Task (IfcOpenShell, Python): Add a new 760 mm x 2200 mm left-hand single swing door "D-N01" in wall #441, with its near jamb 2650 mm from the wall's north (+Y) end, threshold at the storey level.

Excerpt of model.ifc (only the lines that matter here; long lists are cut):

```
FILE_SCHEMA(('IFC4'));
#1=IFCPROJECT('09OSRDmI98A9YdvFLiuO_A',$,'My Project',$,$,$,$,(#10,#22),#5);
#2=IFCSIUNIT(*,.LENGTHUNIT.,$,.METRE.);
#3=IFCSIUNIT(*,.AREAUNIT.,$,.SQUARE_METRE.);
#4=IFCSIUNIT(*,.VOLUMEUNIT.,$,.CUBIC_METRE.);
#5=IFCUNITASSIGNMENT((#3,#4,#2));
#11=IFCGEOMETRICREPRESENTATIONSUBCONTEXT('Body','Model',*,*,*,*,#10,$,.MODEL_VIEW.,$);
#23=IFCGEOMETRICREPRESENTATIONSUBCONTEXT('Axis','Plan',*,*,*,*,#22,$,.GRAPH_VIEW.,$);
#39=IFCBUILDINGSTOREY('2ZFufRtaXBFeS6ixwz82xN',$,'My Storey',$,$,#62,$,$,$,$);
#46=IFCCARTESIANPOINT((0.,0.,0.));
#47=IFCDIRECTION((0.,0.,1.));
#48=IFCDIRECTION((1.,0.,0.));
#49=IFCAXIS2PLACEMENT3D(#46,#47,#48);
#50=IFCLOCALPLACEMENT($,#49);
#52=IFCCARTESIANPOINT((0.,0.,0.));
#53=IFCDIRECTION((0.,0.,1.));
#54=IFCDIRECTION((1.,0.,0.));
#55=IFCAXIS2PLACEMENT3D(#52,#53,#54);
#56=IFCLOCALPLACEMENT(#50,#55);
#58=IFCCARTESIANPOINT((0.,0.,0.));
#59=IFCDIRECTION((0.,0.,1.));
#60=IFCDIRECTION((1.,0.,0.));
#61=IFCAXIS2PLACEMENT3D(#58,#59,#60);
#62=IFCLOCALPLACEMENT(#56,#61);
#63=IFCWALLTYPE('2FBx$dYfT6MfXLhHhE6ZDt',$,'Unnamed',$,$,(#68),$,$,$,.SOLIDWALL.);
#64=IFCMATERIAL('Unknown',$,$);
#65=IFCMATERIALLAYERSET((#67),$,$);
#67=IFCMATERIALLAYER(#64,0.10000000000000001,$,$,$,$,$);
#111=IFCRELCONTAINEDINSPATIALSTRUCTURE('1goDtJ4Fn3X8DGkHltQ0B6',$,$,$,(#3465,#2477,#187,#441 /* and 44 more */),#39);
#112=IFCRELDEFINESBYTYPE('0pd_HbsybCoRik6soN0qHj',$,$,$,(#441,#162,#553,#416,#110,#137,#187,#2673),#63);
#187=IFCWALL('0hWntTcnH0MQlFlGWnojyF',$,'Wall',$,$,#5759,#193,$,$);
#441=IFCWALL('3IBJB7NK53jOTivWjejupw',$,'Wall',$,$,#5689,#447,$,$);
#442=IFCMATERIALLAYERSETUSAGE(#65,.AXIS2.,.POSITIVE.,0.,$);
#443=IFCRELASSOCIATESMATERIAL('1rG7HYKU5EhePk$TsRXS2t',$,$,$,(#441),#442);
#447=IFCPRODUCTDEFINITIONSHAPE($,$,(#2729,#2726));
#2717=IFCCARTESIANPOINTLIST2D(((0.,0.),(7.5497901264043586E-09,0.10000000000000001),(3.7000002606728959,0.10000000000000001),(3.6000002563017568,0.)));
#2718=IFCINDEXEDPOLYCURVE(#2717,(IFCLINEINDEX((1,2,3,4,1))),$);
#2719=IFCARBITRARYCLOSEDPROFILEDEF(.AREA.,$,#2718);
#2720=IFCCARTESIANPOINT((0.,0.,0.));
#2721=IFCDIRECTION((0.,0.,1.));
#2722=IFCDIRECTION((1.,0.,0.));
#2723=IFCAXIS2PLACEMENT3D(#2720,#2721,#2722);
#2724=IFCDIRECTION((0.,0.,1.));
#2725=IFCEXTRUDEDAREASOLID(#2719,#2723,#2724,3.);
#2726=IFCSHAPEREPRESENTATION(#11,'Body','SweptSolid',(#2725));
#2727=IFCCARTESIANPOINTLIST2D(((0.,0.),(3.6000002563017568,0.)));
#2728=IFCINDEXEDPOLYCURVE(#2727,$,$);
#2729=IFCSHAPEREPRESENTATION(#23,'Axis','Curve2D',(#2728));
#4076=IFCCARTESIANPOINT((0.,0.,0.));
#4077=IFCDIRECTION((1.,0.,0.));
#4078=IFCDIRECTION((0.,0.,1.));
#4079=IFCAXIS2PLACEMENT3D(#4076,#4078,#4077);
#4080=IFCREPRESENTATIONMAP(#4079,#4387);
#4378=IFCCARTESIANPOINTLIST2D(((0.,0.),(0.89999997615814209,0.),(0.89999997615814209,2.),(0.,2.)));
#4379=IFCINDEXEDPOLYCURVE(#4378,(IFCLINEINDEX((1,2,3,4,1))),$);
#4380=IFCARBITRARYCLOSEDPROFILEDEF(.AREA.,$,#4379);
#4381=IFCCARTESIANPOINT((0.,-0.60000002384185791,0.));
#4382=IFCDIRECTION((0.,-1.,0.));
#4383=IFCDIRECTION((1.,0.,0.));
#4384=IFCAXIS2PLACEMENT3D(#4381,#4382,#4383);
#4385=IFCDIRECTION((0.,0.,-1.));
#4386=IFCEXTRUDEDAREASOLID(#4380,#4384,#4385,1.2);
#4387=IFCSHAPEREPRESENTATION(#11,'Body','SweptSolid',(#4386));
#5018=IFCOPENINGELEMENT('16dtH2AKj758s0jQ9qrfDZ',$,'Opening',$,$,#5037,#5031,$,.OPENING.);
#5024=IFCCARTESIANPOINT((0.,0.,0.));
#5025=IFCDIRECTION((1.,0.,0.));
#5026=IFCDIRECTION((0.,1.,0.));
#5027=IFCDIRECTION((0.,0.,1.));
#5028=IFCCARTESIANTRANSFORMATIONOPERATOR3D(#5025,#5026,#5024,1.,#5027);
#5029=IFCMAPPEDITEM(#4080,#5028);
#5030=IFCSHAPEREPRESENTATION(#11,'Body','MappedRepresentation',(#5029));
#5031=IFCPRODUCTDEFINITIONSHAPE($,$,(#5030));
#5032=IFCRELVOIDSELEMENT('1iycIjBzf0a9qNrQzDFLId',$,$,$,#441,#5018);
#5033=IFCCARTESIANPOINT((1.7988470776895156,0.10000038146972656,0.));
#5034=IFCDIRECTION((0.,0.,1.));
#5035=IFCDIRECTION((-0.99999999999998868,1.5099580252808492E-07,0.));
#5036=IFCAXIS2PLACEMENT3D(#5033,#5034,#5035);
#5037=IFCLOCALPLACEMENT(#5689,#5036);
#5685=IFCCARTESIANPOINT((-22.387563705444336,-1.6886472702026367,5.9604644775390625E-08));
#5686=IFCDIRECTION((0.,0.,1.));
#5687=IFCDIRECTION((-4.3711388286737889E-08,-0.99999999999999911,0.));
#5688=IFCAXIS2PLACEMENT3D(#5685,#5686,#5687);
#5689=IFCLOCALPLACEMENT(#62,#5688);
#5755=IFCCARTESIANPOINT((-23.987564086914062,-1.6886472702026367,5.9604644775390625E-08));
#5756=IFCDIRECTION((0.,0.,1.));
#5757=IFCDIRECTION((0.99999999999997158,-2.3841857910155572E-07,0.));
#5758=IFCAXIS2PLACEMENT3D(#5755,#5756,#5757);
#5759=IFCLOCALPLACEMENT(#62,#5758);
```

```python
import numpy as np
import ifcopenshell
import ifcopenshell.api.feature
import ifcopenshell.api.geometry
import ifcopenshell.api.root
import ifcopenshell.api.spatial
import ifcopenshell.geom
import ifcopenshell.util.element
import ifcopenshell.util.placement
import ifcopenshell.util.representation
import ifcopenshell.util.shape
import ifcopenshell.util.unit

model = ifcopenshell.open("model.ifc")
unit_scale = ifcopenshell.util.unit.calculate_unit_scale(model)
settings = ifcopenshell.geom.settings()


def volume(element):
    """Net volume in cubic metres, openings subtracted."""
    shape = ifcopenshell.geom.create_shape(settings, element)
    return ifcopenshell.util.shape.get_volume(shape.geometry)


wall = model.by_guid("3IBJB7NK53jOTivWjejupw")
storey = ifcopenshell.util.element.get_container(wall, ifc_class="IfcBuildingStorey")
context = ifcopenshell.util.representation.get_context(model, "Model", "Body", "MODEL_VIEW")
before = volume(wall)

width, height, from_end, sill = 0.76, 2.2, 2.65, 0.0  # metres

# The wall runs along its own X axis, and the end named is its -X end.
wall_shape = ifcopenshell.geom.create_shape(settings, wall)
x, y, z = ifcopenshell.util.shape.get_vertices(wall_shape.geometry).T
start = x.min() + from_end
face, thickness = float(y.min()), float(y.max() - y.min())
wall_matrix = ifcopenshell.util.placement.get_local_placement(wall.ObjectPlacement)
level = ifcopenshell.util.placement.get_local_placement(storey.ObjectPlacement)[2, 3]


def in_wall(x, y):
    """Placement at x, y metres in the wall's axes, at sill height."""
    matrix = wall_matrix.copy()
    matrix[:, 3] = wall_matrix @ np.array([x / unit_scale, y / unit_scale, 0.0, 1.0])
    matrix[2, 3] = level + sill / unit_scale
    return matrix


# Opening: a box that overshoots both wall faces by 50 mm.
opening = ifcopenshell.api.root.create_entity(model, ifc_class="IfcOpeningElement", predefined_type="OPENING")
box = ifcopenshell.api.geometry.add_wall_representation(
    model, context=context, length=width, height=height, thickness=thickness + 0.1
)
ifcopenshell.api.geometry.assign_representation(model, product=opening, representation=box)
ifcopenshell.api.geometry.edit_object_placement(model, product=opening, matrix=in_wall(start, face - 0.05), is_si=False)
ifcopenshell.api.feature.add_feature(model, feature=opening, element=wall)

door = ifcopenshell.api.root.create_entity(model, ifc_class="IfcDoor", name="D-N01", predefined_type="DOOR")
door.OverallWidth, door.OverallHeight = width / unit_scale, height / unit_scale
door.OperationType = "SINGLE_SWING_LEFT"
body = ifcopenshell.api.geometry.add_door_representation(
    model,
    context=context,
    overall_width=door.OverallWidth,
    overall_height=door.OverallHeight,
    operation_type="SINGLE_SWING_LEFT",
    lining_properties={"LiningDepth": thickness / unit_scale, "ThresholdDepth": thickness / unit_scale},
)
ifcopenshell.api.geometry.assign_representation(model, product=door, representation=body)
ifcopenshell.api.spatial.assign_container(model, products=[door], relating_structure=storey)
ifcopenshell.api.feature.add_filling(model, opening=opening, element=door)

# The lining spans the wall, so the door starts at the wall face.
ifcopenshell.api.geometry.edit_object_placement(model, product=door, matrix=in_wall(start, face), is_si=False)

after = volume(wall)

print(f"wall volume {before:.3f} -> {after:.3f} m3")

model.write("model_v2.ifc")
```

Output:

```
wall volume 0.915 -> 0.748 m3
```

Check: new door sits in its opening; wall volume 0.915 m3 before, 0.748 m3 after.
